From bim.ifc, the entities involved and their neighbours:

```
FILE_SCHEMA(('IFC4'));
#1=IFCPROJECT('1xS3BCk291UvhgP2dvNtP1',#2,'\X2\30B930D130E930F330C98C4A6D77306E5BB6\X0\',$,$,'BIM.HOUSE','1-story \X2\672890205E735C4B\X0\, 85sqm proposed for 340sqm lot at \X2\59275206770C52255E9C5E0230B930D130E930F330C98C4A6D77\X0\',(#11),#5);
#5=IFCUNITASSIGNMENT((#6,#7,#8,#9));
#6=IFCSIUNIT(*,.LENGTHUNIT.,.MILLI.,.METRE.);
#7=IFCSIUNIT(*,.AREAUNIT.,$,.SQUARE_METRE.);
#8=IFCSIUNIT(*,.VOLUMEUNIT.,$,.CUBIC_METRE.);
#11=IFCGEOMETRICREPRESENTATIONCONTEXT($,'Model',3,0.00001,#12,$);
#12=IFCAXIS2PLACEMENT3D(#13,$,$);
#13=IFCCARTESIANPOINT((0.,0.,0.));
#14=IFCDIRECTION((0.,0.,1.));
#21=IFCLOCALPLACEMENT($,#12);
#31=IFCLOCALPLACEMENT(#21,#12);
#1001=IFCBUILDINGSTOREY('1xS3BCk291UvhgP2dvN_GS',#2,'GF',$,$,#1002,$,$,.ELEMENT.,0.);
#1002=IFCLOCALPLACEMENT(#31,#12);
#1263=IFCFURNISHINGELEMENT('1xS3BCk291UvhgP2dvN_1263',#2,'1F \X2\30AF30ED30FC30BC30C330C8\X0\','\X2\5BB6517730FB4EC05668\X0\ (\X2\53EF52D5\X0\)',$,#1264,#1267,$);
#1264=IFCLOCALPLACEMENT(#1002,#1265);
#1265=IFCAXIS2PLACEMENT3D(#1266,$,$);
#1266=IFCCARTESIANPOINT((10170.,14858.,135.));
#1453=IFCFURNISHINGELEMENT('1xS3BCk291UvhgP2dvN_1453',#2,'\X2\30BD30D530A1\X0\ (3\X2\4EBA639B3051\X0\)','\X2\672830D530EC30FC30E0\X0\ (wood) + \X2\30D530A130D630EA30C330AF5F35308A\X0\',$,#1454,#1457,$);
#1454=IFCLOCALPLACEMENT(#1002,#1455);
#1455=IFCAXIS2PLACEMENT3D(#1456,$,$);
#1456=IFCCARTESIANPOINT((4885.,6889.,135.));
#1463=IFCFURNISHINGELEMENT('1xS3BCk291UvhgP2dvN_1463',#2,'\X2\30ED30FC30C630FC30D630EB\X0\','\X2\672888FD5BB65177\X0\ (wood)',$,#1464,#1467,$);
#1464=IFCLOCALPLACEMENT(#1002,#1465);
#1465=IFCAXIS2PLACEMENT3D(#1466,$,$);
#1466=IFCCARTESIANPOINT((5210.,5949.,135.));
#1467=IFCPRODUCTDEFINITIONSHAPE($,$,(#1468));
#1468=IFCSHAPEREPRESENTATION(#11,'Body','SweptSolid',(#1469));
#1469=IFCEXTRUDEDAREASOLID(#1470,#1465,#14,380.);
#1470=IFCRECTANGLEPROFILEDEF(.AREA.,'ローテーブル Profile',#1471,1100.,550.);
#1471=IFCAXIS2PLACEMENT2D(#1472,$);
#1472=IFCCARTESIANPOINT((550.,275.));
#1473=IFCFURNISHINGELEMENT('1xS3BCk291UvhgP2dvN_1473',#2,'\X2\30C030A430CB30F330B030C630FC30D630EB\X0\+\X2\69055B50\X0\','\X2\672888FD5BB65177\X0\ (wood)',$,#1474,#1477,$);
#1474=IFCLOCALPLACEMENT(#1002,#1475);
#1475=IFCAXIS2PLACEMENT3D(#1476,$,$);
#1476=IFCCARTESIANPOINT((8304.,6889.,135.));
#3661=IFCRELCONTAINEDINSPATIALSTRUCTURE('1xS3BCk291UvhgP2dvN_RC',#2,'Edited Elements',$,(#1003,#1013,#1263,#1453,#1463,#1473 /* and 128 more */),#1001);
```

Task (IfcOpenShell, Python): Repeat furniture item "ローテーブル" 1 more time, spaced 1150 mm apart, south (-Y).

```python
import numpy as np
import ifcopenshell
import ifcopenshell.api.geometry
import ifcopenshell.api.root
import ifcopenshell.util.element
import ifcopenshell.util.placement

model = ifcopenshell.open("bim.ifc")


def reuse_history(source, copy):
    """copy_class also copies each property set's owner history, people and application; keep the originals."""
    for rel in copy.IsDefinedBy:
        if rel.is_a("IfcRelDefinesByProperties") and (history := rel.RelatingPropertyDefinition.OwnerHistory):
            rel.RelatingPropertyDefinition.OwnerHistory = source.OwnerHistory
            ifcopenshell.util.element.remove_deep2(model, history)


source = model.by_id(1463)
base = ifcopenshell.util.placement.get_local_placement(source.ObjectPlacement)
step = np.array([0.0, -1.0, 0.0]) * 1150.0

for i in range(1, 2):
    copy = ifcopenshell.api.root.copy_class(model, product=source)
    copy.Representation = ifcopenshell.util.element.copy_deep(
        model, source.Representation, exclude=["IfcGeometricRepresentationContext", "IfcRepresentationMap"]
    )
    reuse_history(source, copy)
    matrix = base.copy()
    matrix[:3, 3] += i * step
    print("added at", matrix[:3, 3].round(3) + 0.0)
    ifcopenshell.api.geometry.edit_object_placement(model, product=copy, matrix=matrix, is_si=False)

model.write("bim_edited.ifc")
```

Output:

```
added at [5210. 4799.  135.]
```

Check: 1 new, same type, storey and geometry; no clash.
